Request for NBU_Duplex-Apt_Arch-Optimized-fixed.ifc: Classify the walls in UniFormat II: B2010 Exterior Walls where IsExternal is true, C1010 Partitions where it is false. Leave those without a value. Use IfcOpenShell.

First a look at what the model holds.

```python
import ifcopenshell
import ifcopenshell.util.element

model = ifcopenshell.open("NBU_Duplex-Apt_Arch-Optimized-fixed.ifc")
print(model.schema)
print("classifications:", [c.Name for c in model.by_type("IfcClassification")])
values = [ifcopenshell.util.element.get_pset(e, "Pset_WallCommon", "IsExternal") for e in model.by_type("IfcWall")]
for value in (True, False, None):
    print("IsExternal", value, values.count(value))
```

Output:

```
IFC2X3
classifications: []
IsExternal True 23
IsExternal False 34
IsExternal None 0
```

```python
import ifcopenshell
import ifcopenshell.api.classification
import ifcopenshell.util.element

model = ifcopenshell.open("NBU_Duplex-Apt_Arch-Optimized-fixed.ifc")

# IFC2X3 requires Source and Edition and has no link from the project to the system.
system = model.create_entity("IfcClassification", Source="ASTM", Edition="E1557", Name="UniFormat II")

walls = model.by_type("IfcWall")
external = {e: ifcopenshell.util.element.get_pset(e, "Pset_WallCommon", "IsExternal") for e in walls}
for flag, code, name in ((True, "B2010", "Exterior Walls"), (False, "C1010", "Partitions")):
    products = [e for e in walls if external[e] is flag]
    ifcopenshell.api.classification.add_reference(
        model, products=products, classification=system, identification=code, name=name
    )
    print(code, len(products))

model.write("NBU_Duplex-Apt_Arch-Optimized-fixed_edited.ifc")
```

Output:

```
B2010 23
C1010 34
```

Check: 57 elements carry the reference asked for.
